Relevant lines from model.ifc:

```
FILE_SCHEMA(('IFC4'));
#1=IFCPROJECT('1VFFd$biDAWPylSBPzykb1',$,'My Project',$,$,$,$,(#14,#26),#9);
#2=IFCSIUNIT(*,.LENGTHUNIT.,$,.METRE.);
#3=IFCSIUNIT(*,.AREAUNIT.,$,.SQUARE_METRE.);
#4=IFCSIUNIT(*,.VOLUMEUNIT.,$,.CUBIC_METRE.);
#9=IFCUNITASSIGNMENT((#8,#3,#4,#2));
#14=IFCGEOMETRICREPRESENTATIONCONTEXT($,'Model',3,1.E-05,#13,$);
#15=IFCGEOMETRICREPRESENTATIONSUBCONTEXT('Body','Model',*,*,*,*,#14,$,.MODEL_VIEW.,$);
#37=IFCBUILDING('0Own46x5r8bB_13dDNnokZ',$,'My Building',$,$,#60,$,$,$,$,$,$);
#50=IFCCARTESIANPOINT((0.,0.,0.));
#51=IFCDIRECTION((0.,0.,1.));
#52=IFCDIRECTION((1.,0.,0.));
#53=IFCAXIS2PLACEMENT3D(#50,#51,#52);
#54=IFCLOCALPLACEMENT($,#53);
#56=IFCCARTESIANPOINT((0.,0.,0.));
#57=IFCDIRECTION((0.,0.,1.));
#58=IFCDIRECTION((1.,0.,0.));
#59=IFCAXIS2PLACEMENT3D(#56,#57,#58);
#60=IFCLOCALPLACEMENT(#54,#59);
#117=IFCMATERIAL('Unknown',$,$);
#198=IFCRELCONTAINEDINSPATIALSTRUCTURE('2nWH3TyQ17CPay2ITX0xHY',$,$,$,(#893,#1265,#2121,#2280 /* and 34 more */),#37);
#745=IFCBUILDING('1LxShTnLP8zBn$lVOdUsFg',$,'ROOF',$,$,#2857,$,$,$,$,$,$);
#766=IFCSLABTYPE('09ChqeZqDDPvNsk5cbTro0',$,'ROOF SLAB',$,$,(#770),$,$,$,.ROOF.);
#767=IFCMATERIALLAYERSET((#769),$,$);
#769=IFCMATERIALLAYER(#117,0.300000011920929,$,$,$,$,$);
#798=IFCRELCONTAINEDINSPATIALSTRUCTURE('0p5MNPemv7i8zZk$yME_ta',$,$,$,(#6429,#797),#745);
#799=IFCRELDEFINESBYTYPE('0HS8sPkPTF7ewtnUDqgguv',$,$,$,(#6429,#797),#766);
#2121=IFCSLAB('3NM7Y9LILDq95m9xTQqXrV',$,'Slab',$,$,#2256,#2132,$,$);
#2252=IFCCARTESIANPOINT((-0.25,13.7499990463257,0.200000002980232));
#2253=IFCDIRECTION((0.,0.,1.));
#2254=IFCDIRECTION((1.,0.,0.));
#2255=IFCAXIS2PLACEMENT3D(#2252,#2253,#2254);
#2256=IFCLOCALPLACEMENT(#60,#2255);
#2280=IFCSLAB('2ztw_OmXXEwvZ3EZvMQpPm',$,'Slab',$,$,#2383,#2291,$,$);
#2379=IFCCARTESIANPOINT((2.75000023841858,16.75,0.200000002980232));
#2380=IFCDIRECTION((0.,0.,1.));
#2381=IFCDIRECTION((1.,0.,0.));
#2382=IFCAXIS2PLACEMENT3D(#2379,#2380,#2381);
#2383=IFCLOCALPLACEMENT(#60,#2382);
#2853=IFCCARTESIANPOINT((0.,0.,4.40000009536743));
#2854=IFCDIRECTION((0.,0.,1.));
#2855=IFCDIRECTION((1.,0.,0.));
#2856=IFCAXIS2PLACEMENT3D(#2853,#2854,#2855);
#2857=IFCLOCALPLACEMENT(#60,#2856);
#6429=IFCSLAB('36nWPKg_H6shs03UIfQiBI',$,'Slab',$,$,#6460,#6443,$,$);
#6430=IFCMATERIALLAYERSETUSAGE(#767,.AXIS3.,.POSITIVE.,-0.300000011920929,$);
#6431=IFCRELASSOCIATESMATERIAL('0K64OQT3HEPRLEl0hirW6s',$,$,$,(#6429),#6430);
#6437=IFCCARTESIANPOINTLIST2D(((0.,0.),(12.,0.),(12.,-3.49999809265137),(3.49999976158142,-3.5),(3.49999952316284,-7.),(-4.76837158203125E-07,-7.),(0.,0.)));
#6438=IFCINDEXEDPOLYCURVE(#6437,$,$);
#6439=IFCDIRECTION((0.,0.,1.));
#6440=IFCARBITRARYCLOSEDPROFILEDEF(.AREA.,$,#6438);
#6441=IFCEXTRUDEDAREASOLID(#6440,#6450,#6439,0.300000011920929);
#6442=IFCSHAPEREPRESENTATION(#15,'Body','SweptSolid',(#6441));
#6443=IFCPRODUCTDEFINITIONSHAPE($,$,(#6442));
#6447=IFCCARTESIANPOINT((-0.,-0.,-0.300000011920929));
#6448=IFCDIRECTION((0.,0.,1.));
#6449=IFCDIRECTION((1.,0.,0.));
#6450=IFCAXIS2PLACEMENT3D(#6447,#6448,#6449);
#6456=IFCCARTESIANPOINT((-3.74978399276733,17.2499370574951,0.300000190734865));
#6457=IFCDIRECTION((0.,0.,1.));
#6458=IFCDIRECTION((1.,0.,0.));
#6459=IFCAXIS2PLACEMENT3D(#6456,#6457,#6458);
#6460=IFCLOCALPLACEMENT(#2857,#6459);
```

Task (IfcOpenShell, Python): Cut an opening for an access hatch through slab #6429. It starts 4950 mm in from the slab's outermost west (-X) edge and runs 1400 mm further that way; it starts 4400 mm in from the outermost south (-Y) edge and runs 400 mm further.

```python
import numpy as np
import ifcopenshell
import ifcopenshell.api.feature
import ifcopenshell.api.geometry
import ifcopenshell.api.root
import ifcopenshell.geom
import ifcopenshell.util.placement
import ifcopenshell.util.representation
import ifcopenshell.util.shape
import ifcopenshell.util.unit

model = ifcopenshell.open("model.ifc")
unit_scale = ifcopenshell.util.unit.calculate_unit_scale(model)
settings = ifcopenshell.geom.settings()


def volume(element):
    """Net volume in cubic metres, openings subtracted."""
    shape = ifcopenshell.geom.create_shape(settings, element)
    return ifcopenshell.util.shape.get_volume(shape.geometry)


slab = model.by_id(6429)
before = volume(slab)

# Extent in the slab's own axes, in metres. The edges named are its -X and -Y sides.
slab_shape = ifcopenshell.geom.create_shape(settings, slab)
vertices = ifcopenshell.util.shape.get_vertices(slab_shape.geometry)
x_min, y_min, bottom = vertices.min(axis=0)
top = vertices[:, 2].max()

opening = ifcopenshell.api.root.create_entity(model, ifc_class="IfcOpeningElement", name="Access hatch opening", predefined_type="OPENING")
context = ifcopenshell.util.representation.get_context(model, "Model", "Body", "MODEL_VIEW")
width, depth = 1.4, 0.4
outline = [(0.0, 0.0), (width, 0.0), (width, depth), (0.0, depth), (0.0, 0.0)]
# Overshoot both faces by 50 mm so the cut is clean.
shape = ifcopenshell.api.geometry.add_slab_representation(
    model, context=context, depth=top - bottom + 0.1, polyline=outline
)
ifcopenshell.api.geometry.assign_representation(model, product=opening, representation=shape)

matrix = ifcopenshell.util.placement.get_local_placement(slab.ObjectPlacement)
matrix[:, 3] = matrix @ np.append(np.array([x_min + 4.95, y_min + 4.4, bottom - 0.05]) / unit_scale, 1.0)
ifcopenshell.api.geometry.edit_object_placement(model, product=opening, matrix=matrix, is_si=False)
ifcopenshell.api.feature.add_feature(model, feature=opening, element=slab)

after = volume(slab)

print(f"slab volume {before:.3f} -> {after:.3f} m3")

model.write("model-out.ifc")
```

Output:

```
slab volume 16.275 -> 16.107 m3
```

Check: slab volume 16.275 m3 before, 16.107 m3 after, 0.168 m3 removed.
